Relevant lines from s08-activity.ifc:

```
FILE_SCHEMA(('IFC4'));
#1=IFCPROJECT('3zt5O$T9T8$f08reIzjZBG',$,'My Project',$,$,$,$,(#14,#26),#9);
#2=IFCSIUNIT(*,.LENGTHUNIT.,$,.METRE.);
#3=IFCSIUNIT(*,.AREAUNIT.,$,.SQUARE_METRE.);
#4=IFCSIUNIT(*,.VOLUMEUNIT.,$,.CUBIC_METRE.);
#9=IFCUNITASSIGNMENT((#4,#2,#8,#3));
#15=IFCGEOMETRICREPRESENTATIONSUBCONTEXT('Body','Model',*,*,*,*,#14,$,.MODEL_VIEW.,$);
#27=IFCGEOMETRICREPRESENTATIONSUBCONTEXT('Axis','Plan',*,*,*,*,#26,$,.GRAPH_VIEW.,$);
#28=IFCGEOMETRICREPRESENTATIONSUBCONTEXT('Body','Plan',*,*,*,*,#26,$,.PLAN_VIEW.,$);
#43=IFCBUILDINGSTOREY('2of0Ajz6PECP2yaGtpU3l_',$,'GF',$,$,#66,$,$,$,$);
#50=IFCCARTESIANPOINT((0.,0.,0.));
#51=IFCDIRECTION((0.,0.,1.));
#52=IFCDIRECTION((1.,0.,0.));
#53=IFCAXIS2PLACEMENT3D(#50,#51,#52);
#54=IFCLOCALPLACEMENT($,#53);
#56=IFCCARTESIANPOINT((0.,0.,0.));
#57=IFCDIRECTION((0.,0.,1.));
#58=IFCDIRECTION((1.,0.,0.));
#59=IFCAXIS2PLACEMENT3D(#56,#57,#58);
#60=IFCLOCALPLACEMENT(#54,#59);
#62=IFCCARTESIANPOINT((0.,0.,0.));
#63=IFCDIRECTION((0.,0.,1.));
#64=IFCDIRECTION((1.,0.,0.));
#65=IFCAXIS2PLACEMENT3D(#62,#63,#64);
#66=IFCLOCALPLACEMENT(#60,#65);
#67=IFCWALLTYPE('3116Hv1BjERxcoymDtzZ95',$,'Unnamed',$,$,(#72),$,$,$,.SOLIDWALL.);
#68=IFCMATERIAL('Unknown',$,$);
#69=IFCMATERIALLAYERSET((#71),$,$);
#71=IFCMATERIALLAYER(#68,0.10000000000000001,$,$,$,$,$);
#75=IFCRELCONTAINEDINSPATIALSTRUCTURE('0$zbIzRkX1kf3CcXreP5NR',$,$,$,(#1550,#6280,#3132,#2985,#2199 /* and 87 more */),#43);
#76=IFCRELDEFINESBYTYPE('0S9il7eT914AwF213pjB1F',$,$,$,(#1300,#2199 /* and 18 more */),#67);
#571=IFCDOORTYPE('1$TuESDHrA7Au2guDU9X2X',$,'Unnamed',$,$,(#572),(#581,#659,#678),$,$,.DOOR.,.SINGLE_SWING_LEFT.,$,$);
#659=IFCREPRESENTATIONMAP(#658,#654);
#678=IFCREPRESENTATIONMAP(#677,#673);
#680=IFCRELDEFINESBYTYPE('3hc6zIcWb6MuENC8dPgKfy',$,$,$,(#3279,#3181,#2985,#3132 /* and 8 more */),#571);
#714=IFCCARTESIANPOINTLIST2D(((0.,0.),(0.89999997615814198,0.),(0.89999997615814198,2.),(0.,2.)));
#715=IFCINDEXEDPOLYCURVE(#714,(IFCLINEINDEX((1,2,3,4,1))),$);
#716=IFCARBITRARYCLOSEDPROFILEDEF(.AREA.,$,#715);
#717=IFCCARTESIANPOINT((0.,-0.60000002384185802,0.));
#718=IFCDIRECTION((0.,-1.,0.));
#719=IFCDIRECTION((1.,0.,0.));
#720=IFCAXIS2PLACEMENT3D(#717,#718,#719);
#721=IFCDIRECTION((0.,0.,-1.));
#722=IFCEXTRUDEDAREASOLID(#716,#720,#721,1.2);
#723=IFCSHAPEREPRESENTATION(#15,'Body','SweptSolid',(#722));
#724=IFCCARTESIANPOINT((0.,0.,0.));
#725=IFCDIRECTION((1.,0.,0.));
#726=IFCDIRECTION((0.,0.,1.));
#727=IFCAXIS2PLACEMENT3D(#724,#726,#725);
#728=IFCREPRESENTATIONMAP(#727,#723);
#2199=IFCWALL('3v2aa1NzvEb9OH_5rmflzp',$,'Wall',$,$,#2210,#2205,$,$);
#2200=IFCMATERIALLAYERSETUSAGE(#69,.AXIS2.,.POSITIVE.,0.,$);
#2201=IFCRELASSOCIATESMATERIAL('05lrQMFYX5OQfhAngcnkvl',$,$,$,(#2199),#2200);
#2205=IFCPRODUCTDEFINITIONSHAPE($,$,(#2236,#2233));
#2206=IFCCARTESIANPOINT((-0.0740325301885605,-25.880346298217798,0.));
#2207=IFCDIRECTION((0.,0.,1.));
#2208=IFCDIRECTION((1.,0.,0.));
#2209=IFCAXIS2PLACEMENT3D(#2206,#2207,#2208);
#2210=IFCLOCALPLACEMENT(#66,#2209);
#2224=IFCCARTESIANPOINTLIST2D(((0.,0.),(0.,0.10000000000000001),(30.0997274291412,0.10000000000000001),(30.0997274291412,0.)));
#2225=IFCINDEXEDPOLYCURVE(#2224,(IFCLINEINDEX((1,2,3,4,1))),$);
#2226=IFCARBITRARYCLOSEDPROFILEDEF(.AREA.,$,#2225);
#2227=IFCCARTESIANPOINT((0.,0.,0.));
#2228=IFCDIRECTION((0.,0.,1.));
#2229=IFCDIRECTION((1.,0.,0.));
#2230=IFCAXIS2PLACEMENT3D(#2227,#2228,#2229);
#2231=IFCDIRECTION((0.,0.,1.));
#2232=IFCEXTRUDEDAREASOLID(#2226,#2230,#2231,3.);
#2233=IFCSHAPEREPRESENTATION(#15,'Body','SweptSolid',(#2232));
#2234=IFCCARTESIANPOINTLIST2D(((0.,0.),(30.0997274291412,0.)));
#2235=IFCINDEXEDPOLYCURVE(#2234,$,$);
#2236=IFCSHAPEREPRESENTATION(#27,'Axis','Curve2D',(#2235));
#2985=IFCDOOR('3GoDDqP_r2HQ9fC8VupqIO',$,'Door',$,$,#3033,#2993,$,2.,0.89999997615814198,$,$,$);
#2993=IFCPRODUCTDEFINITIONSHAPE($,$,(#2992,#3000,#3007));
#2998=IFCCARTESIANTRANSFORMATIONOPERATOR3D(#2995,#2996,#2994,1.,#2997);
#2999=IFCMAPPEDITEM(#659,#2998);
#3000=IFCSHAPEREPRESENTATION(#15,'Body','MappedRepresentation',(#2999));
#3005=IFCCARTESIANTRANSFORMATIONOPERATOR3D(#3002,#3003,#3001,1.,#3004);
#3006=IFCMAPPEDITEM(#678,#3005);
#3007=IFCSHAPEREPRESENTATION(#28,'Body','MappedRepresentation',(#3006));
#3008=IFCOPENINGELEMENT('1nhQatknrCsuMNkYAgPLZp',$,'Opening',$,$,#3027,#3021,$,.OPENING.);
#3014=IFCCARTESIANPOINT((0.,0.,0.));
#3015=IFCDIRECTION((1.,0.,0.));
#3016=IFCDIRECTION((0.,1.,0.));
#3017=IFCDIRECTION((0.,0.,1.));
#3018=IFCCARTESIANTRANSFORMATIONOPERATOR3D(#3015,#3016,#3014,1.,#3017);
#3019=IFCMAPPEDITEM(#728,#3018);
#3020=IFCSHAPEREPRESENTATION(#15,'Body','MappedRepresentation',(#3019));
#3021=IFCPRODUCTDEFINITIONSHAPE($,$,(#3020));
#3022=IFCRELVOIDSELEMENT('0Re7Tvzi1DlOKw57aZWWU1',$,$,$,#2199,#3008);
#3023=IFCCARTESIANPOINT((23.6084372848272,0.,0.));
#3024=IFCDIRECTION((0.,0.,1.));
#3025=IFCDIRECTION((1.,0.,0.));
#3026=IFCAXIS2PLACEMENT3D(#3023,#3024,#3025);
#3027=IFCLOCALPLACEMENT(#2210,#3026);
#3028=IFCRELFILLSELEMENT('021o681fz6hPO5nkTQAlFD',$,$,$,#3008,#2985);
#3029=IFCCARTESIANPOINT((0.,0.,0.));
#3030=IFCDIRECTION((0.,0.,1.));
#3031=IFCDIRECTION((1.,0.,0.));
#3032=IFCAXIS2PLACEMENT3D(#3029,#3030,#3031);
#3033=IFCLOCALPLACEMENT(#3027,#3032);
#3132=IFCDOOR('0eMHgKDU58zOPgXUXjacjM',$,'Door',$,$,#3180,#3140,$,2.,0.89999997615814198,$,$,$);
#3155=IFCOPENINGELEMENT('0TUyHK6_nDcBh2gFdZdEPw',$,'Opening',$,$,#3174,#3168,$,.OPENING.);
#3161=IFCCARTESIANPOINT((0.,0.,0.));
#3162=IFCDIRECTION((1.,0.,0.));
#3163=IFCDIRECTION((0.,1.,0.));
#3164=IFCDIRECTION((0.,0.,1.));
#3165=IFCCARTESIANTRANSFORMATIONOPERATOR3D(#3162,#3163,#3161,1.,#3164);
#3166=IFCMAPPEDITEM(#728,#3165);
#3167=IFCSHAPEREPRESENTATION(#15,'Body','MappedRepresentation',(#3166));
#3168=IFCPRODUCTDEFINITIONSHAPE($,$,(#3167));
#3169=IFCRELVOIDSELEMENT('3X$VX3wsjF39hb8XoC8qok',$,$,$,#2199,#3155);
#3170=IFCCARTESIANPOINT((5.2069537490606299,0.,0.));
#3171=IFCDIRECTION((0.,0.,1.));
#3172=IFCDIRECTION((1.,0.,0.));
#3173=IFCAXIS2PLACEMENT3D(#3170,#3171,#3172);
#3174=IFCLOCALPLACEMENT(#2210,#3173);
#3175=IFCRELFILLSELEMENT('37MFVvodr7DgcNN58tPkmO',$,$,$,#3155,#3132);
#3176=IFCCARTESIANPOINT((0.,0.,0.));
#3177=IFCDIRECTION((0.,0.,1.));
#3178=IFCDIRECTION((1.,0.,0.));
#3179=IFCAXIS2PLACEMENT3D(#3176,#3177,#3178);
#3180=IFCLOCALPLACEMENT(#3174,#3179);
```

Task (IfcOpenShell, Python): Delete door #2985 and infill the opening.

```python
import ifcopenshell
import ifcopenshell.api.feature
import ifcopenshell.api.root
import ifcopenshell.geom
import ifcopenshell.util.shape

model = ifcopenshell.open("s08-activity.ifc")
settings = ifcopenshell.geom.settings()


def volume(element):
    """Net volume in cubic metres, openings subtracted."""
    shape = ifcopenshell.geom.create_shape(settings, element)
    return ifcopenshell.util.shape.get_volume(shape.geometry)


door = model.by_guid("3GoDDqP_r2HQ9fC8VupqIO")
opening = door.FillsVoids[0].RelatingOpeningElement
wall = opening.VoidsElements[0].RelatingBuildingElement
before = volume(wall)

ifcopenshell.api.root.remove_product(model, product=door)
ifcopenshell.api.feature.remove_feature(model, feature=opening)

after = volume(wall)

print(f"wall volume {before:.3f} -> {after:.3f} m3")

model.write("s08-activity_rev.ifc")
```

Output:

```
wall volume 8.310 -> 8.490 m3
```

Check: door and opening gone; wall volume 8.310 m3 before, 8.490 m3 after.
